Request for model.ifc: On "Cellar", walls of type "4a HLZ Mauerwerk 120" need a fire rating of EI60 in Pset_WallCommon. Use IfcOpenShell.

First a look at what the model holds.

```python
import ifcopenshell
import ifcopenshell.util.element

model = ifcopenshell.open("model.ifc")
print(model.schema)
storey = next(s for s in model.by_type("IfcBuildingStorey") if s.Name == "Cellar")
walls = [e for e in ifcopenshell.util.element.get_decomposition(storey) if e.is_a("IfcWall")]
seen = {}
for e in walls:
    element_type = ifcopenshell.util.element.get_type(e)
    key = (element_type.Name if element_type != e and element_type else None, ifcopenshell.util.element.get_pset(e, "Pset_WallCommon", "FireRating"))
    seen[key] = seen.get(key, 0) + 1
for (name, value), count in sorted(seen.items(), key=str):
    print(count, "x", name, "|", value)
```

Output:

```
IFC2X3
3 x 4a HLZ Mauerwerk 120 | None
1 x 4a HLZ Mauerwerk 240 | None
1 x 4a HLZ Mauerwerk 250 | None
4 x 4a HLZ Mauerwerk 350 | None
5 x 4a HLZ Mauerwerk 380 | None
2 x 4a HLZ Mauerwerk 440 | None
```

```python
import ifcopenshell
import ifcopenshell.api.pset
import ifcopenshell.util.element

model = ifcopenshell.open("model.ifc")

storey = next(s for s in model.by_type("IfcBuildingStorey") if s.Name == "Cellar")
walls = [e for e in ifcopenshell.util.element.get_decomposition(storey) if e.is_a("IfcWall")]

count = 0
for e in walls:
    element_type = ifcopenshell.util.element.get_type(e)
    if element_type in (None, e) or element_type.Name != "4a HLZ Mauerwerk 120":
        continue
    # add_pset returns the element's existing set when there is one.
    pset = ifcopenshell.api.pset.add_pset(model, product=e, name="Pset_WallCommon")
    ifcopenshell.api.pset.edit_pset(model, pset=pset, properties={"FireRating": "EI60"})
    count += 1

print(count, "walls updated")

model.write("model_rev.ifc")
```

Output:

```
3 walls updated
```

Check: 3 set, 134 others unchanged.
